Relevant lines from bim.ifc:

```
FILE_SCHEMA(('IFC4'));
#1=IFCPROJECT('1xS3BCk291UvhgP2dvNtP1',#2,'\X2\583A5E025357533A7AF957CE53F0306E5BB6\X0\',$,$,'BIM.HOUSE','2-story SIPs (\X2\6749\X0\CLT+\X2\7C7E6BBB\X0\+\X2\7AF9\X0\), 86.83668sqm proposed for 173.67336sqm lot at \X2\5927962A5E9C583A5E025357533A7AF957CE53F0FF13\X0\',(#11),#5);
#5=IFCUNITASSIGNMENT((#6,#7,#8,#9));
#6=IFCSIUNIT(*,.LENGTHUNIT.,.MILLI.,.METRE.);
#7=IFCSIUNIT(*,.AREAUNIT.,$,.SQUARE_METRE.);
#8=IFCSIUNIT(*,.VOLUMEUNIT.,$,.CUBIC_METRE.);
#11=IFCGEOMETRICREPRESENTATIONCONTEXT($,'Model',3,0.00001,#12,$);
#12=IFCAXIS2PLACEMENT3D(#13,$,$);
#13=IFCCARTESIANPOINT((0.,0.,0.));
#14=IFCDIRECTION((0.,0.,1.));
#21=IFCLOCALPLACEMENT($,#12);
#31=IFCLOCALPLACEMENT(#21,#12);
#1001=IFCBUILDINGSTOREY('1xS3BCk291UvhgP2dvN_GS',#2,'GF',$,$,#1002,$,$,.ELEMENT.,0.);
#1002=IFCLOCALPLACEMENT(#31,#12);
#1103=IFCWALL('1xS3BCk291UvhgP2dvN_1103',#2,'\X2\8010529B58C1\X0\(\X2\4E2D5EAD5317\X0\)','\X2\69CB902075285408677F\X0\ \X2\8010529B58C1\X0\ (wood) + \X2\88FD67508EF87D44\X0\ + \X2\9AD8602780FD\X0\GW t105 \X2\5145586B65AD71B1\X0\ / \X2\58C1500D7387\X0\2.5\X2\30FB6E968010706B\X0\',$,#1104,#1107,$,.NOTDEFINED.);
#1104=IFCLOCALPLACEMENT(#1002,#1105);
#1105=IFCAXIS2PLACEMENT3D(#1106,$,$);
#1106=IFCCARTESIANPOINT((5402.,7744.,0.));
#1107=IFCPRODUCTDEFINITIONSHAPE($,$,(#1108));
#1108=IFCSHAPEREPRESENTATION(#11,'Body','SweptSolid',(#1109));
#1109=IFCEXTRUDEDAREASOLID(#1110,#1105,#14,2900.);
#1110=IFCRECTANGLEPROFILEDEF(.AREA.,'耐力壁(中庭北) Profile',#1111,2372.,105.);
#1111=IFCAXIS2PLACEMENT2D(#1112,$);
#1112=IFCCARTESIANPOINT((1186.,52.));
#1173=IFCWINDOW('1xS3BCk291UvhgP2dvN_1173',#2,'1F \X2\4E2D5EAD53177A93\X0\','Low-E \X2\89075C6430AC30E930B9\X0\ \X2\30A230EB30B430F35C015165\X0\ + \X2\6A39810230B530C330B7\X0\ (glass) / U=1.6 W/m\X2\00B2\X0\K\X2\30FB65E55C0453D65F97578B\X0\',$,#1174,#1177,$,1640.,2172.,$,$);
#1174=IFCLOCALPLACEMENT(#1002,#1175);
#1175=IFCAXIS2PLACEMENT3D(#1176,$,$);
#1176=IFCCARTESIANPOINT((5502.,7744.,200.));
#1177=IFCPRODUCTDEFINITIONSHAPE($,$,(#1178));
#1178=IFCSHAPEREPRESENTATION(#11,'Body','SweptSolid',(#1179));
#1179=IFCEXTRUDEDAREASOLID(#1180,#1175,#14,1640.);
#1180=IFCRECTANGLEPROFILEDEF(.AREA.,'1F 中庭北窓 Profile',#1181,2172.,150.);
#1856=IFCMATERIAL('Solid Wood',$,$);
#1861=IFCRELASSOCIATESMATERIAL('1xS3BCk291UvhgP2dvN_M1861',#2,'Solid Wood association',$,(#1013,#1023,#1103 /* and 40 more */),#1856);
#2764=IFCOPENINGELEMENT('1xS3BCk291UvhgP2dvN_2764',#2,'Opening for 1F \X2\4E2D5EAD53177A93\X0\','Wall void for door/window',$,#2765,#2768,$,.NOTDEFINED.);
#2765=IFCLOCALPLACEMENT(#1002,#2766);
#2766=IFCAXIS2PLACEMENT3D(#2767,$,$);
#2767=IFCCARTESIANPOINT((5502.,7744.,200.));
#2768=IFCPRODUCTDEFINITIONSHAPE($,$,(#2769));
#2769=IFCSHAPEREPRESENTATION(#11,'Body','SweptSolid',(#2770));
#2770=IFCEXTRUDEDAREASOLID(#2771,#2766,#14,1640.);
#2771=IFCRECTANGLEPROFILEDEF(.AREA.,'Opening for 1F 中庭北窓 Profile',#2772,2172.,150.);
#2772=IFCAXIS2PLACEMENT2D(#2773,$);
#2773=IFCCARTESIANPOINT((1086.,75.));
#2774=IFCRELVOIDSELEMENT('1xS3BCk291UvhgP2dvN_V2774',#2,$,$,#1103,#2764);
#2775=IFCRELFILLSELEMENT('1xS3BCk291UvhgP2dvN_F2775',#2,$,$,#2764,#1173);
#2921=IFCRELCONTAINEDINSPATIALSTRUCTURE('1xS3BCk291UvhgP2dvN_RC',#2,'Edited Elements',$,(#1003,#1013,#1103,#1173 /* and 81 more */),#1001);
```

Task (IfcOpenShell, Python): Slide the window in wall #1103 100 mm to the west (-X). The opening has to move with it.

```python
import ifcopenshell
import ifcopenshell.api.geometry
import ifcopenshell.util.placement

model = ifcopenshell.open("bim.ifc")

window = model.by_guid("1xS3BCk291UvhgP2dvN_1173")
opening = window.FillsVoids[0].RelatingOpeningElement
wall = opening.VoidsElements[0].RelatingBuildingElement

wall_matrix = ifcopenshell.util.placement.get_local_placement(wall.ObjectPlacement)
shift = wall_matrix[:3, 0] * -100.0
before = ifcopenshell.util.placement.get_local_placement(window.ObjectPlacement)[:3, 3].copy()

# The window is not placed relative to its opening, so move both.
for product in (opening, window):
    matrix = ifcopenshell.util.placement.get_local_placement(product.ObjectPlacement)
    matrix[:3, 3] += shift
    ifcopenshell.api.geometry.edit_object_placement(model, product=product, matrix=matrix, is_si=False)

after = ifcopenshell.util.placement.get_local_placement(window.ObjectPlacement)[:3, 3]
print("window moved by", (after - before).round(3) + 0.0)

model.write("bim_v2.ifc")
```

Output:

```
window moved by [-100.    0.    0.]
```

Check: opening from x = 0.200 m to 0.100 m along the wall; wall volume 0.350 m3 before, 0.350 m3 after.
